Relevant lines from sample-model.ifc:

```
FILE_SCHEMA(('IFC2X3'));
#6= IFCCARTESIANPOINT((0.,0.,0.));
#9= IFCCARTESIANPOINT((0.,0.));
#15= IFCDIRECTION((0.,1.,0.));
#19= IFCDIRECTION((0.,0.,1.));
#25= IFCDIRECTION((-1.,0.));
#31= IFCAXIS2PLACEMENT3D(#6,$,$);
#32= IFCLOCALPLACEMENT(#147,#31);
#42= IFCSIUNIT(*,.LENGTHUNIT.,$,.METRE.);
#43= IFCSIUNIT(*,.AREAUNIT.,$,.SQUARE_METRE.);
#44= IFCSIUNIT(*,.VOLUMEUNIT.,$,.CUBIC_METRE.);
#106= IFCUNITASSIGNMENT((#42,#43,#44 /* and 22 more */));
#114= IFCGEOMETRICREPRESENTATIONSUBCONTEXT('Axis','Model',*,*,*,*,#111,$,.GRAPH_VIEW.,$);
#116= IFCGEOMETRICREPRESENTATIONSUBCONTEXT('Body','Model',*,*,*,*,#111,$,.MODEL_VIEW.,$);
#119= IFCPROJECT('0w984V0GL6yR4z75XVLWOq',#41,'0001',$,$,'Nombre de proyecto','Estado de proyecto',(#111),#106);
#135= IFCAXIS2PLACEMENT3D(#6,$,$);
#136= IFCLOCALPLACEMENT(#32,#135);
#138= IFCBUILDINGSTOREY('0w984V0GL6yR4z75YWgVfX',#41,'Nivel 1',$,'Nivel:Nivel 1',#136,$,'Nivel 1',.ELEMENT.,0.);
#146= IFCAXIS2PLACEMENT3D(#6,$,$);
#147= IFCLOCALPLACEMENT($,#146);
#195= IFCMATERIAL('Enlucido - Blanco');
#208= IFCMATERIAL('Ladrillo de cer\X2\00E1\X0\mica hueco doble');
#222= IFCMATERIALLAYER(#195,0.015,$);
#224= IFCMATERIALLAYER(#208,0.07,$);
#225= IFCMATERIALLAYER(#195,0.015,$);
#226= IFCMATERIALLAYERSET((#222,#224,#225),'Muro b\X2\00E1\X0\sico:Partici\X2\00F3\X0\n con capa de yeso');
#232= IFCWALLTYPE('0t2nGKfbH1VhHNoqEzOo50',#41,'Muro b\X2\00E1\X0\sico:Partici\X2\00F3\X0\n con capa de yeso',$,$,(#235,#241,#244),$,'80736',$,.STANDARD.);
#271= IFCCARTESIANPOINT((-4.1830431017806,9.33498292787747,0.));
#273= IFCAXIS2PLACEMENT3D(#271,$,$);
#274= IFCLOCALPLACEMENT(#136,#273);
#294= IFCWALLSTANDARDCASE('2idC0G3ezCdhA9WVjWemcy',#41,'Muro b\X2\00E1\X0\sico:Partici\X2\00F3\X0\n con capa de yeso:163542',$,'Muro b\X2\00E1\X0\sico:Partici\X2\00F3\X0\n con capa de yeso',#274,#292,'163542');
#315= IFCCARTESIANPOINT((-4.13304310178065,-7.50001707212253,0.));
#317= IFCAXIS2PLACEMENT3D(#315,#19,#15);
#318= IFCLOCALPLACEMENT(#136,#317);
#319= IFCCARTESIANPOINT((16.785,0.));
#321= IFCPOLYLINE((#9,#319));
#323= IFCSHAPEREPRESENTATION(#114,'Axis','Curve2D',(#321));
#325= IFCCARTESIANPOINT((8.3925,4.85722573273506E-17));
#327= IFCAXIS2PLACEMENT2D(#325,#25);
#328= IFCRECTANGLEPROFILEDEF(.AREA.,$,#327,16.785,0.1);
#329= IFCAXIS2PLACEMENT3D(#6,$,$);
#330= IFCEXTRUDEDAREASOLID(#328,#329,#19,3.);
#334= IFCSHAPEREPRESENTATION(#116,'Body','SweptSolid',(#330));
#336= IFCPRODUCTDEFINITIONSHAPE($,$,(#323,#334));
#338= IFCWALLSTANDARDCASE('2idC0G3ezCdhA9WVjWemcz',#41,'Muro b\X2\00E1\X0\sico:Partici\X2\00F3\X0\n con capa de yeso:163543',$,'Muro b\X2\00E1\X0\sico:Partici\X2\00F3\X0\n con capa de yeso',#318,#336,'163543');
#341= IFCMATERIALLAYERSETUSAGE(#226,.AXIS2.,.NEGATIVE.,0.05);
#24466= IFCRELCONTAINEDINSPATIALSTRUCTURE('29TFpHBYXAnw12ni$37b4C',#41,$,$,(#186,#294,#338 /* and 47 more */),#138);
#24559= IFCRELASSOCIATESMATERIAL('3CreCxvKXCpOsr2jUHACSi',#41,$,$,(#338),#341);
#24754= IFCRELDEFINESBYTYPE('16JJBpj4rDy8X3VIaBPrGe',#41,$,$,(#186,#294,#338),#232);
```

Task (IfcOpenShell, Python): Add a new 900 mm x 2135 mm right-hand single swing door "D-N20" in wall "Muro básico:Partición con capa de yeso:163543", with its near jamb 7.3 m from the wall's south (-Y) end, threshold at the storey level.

```python
import numpy as np
import ifcopenshell
import ifcopenshell.api.feature
import ifcopenshell.api.geometry
import ifcopenshell.api.root
import ifcopenshell.api.spatial
import ifcopenshell.api.type
import ifcopenshell.geom
import ifcopenshell.util.element
import ifcopenshell.util.placement
import ifcopenshell.util.representation
import ifcopenshell.util.shape
import ifcopenshell.util.unit

model = ifcopenshell.open("sample-model.ifc")
unit_scale = ifcopenshell.util.unit.calculate_unit_scale(model)
settings = ifcopenshell.geom.settings()


def volume(element):
    """Net volume in cubic metres, openings subtracted."""
    shape = ifcopenshell.geom.create_shape(settings, element)
    return ifcopenshell.util.shape.get_volume(shape.geometry)


wall = model.by_guid("2idC0G3ezCdhA9WVjWemcz")
storey = ifcopenshell.util.element.get_container(wall, ifc_class="IfcBuildingStorey")
context = ifcopenshell.util.representation.get_context(model, "Model", "Body", "MODEL_VIEW")
before = volume(wall)

width, height, from_end, sill = 0.9, 2.135, 7.3, 0.0  # metres

# The wall runs along its own X axis, and the end named is its -X end.
wall_shape = ifcopenshell.geom.create_shape(settings, wall)
x, y, z = ifcopenshell.util.shape.get_vertices(wall_shape.geometry).T
start = x.min() + from_end
face, thickness = float(y.min()), float(y.max() - y.min())
wall_matrix = ifcopenshell.util.placement.get_local_placement(wall.ObjectPlacement)
level = ifcopenshell.util.placement.get_local_placement(storey.ObjectPlacement)[2, 3]


def in_wall(x, y):
    """Placement at x, y metres in the wall's axes, at sill height."""
    matrix = wall_matrix.copy()
    matrix[:, 3] = wall_matrix @ np.array([x / unit_scale, y / unit_scale, 0.0, 1.0])
    matrix[2, 3] = level + sill / unit_scale
    return matrix


# Opening: a box that overshoots both wall faces by 50 mm.
opening = ifcopenshell.api.root.create_entity(model, ifc_class="IfcOpeningElement")
box = ifcopenshell.api.geometry.add_wall_representation(
    model, context=context, length=width, height=height, thickness=thickness + 0.1
)
ifcopenshell.api.geometry.assign_representation(model, product=opening, representation=box)
ifcopenshell.api.geometry.edit_object_placement(model, product=opening, matrix=in_wall(start, face - 0.05), is_si=False)
ifcopenshell.api.feature.add_feature(model, feature=opening, element=wall)

door = ifcopenshell.api.root.create_entity(model, ifc_class="IfcDoor", name="D-N20")
door.OverallWidth, door.OverallHeight = width / unit_scale, height / unit_scale
body = ifcopenshell.api.geometry.add_door_representation(
    model,
    context=context,
    overall_width=door.OverallWidth,
    overall_height=door.OverallHeight,
    operation_type="SINGLE_SWING_RIGHT",
    lining_properties={"LiningDepth": thickness / unit_scale, "ThresholdDepth": thickness / unit_scale},
)
ifcopenshell.api.geometry.assign_representation(model, product=door, representation=body)
ifcopenshell.api.spatial.assign_container(model, products=[door], relating_structure=storey)
fills = ifcopenshell.api.feature.add_filling(model, opening=opening, element=door)
fills.OwnerHistory = door.OwnerHistory  # required in IFC2X3

# IFC2X3 keeps the operation on the door style.
style = ifcopenshell.api.root.create_entity(model, ifc_class="IfcDoorStyle", name="D-N20")
style.OperationType, style.ConstructionType = "SINGLE_SWING_RIGHT", "NOTDEFINED"
style.ParameterTakesPrecedence = style.Sizeable = False
ifcopenshell.api.type.assign_type(model, related_objects=[door], relating_type=style)

# The lining spans the wall, so the door starts at the wall face.
ifcopenshell.api.geometry.edit_object_placement(model, product=door, matrix=in_wall(start, face), is_si=False)

after = volume(wall)

print(f"wall volume {before:.3f} -> {after:.3f} m3")

model.write("sample-model_rev.ifc")
```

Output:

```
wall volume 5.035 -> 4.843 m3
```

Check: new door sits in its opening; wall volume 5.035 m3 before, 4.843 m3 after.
